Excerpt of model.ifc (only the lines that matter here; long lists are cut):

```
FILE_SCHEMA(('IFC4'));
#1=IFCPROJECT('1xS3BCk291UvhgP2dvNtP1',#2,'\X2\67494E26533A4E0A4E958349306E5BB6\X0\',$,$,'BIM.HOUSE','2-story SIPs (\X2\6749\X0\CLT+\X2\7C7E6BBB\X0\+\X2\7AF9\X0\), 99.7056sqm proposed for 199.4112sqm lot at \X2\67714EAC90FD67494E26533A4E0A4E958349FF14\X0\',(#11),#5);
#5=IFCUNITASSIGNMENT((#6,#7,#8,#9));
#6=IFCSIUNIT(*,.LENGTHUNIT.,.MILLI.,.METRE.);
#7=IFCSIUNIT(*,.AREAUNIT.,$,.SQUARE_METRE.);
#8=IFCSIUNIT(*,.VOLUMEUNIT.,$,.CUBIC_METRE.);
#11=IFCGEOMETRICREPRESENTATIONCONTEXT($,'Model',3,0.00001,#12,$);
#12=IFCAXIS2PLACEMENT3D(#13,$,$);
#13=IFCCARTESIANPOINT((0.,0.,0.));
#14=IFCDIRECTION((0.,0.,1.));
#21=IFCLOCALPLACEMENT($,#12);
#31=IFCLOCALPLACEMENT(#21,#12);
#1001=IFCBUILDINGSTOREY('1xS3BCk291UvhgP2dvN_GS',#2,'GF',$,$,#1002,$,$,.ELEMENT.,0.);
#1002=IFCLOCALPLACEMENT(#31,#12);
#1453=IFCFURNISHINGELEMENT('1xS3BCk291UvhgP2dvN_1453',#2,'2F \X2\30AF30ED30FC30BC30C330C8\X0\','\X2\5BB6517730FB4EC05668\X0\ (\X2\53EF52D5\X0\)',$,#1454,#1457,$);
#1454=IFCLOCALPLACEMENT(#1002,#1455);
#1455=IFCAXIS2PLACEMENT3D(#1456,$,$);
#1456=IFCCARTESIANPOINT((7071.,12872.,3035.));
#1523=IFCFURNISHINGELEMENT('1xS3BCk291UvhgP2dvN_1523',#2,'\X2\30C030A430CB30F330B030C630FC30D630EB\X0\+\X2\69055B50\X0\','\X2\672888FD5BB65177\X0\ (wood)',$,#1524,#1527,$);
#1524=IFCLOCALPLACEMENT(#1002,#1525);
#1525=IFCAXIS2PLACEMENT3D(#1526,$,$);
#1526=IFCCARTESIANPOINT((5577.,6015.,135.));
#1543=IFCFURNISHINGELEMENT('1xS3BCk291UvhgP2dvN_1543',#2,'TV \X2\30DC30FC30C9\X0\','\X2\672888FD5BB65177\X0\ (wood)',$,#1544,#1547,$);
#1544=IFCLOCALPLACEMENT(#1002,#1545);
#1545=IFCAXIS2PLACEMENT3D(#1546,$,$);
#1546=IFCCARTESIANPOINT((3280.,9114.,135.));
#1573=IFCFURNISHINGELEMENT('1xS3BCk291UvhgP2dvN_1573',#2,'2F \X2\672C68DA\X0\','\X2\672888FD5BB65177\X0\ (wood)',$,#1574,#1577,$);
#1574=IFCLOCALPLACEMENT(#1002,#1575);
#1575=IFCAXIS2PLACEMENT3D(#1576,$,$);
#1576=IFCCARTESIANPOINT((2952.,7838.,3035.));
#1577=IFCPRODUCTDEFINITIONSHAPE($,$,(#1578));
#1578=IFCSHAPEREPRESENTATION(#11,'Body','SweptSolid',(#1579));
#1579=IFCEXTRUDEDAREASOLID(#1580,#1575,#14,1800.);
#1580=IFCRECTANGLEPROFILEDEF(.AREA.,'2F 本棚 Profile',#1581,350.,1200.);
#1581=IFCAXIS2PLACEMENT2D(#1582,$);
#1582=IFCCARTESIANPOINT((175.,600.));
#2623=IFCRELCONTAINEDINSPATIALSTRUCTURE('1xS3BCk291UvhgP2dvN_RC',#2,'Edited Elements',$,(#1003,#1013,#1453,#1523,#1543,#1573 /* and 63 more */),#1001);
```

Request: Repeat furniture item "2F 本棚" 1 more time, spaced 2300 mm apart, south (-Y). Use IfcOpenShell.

```python
import numpy as np
import ifcopenshell
import ifcopenshell.api.geometry
import ifcopenshell.api.root
import ifcopenshell.util.element
import ifcopenshell.util.placement

model = ifcopenshell.open("model.ifc")


def reuse_history(source, copy):
    """copy_class also copies each property set's owner history, people and application; keep the originals."""
    for rel in copy.IsDefinedBy:
        if rel.is_a("IfcRelDefinesByProperties") and (history := rel.RelatingPropertyDefinition.OwnerHistory):
            rel.RelatingPropertyDefinition.OwnerHistory = source.OwnerHistory
            ifcopenshell.util.element.remove_deep2(model, history)


source = model.by_id(1573)
base = ifcopenshell.util.placement.get_local_placement(source.ObjectPlacement)
step = np.array([0.0, -1.0, 0.0]) * 2300.0

for i in range(1, 2):
    copy = ifcopenshell.api.root.copy_class(model, product=source)
    copy.Representation = ifcopenshell.util.element.copy_deep(
        model, source.Representation, exclude=["IfcGeometricRepresentationContext", "IfcRepresentationMap"]
    )
    reuse_history(source, copy)
    matrix = base.copy()
    matrix[:3, 3] += i * step
    print("added at", matrix[:3, 3].round(3) + 0.0)
    ifcopenshell.api.geometry.edit_object_placement(model, product=copy, matrix=matrix, is_si=False)

model.write("model-out.ifc")
```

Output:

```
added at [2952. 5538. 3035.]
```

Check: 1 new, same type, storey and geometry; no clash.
